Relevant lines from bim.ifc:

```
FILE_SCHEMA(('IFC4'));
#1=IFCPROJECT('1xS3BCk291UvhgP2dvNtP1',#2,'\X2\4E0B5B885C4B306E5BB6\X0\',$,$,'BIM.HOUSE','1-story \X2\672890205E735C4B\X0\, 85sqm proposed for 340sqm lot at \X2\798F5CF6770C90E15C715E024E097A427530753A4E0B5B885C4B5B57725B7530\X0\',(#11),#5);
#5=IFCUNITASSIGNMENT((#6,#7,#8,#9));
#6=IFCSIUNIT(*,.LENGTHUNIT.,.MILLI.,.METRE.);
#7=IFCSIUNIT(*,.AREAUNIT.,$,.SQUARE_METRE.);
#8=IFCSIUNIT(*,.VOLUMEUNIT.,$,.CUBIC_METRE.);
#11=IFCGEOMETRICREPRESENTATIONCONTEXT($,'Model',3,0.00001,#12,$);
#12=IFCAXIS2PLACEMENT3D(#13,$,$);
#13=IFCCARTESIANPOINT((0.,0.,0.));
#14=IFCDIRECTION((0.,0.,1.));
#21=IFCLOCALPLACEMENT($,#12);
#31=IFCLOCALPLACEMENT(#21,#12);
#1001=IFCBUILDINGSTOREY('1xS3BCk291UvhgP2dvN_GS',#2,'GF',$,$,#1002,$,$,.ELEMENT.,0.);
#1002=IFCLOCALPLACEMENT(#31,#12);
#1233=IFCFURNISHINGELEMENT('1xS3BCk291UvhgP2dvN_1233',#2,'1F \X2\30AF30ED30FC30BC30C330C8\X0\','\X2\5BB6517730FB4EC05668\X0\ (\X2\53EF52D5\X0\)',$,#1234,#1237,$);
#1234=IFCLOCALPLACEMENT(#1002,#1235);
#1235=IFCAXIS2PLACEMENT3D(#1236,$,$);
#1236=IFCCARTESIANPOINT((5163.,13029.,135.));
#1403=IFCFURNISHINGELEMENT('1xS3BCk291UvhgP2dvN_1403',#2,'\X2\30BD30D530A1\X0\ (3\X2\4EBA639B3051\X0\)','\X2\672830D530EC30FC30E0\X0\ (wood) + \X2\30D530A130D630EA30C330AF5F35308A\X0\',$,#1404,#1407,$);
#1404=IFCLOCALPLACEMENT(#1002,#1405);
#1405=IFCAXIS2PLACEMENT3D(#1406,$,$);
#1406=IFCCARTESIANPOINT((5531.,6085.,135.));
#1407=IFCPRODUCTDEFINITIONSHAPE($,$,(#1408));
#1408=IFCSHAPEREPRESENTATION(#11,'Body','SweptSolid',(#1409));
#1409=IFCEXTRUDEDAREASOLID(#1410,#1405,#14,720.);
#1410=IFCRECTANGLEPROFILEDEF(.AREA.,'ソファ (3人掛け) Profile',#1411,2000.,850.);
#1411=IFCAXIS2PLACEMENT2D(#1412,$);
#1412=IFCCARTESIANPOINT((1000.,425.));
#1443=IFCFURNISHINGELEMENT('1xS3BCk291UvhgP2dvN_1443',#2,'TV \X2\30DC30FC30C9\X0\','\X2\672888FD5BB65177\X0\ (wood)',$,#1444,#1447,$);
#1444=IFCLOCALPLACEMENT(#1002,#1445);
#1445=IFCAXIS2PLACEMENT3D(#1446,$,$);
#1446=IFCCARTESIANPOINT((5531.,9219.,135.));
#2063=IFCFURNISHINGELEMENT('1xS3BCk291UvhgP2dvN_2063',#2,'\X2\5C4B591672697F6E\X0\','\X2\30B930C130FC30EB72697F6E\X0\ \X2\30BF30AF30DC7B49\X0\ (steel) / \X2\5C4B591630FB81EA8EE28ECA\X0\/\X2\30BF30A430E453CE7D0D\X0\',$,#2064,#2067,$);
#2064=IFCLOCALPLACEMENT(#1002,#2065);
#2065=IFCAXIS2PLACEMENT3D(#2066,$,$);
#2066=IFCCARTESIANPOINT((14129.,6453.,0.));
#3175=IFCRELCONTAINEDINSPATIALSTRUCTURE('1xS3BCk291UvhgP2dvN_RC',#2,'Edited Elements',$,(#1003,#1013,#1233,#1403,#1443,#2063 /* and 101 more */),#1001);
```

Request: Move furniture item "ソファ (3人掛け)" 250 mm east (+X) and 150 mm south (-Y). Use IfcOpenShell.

```python
import ifcopenshell
import ifcopenshell.api.geometry
import ifcopenshell.util.placement
import ifcopenshell.util.unit

model = ifcopenshell.open("bim.ifc")
unit_scale = ifcopenshell.util.unit.calculate_unit_scale(model)

item = model.by_id(1403)
matrix = ifcopenshell.util.placement.get_local_placement(item.ObjectPlacement)
matrix[0, 3] += 0.25 / unit_scale
matrix[1, 3] -= 0.15 / unit_scale
ifcopenshell.api.geometry.edit_object_placement(model, product=item, matrix=matrix, is_si=False)

print(ifcopenshell.util.placement.get_local_placement(item.ObjectPlacement).round(3) + 0.0)

model.write("bim_updated.ifc")
```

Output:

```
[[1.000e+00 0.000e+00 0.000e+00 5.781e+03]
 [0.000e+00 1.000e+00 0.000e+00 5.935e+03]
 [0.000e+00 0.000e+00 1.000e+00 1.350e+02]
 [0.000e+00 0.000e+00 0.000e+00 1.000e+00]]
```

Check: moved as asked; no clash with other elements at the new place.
